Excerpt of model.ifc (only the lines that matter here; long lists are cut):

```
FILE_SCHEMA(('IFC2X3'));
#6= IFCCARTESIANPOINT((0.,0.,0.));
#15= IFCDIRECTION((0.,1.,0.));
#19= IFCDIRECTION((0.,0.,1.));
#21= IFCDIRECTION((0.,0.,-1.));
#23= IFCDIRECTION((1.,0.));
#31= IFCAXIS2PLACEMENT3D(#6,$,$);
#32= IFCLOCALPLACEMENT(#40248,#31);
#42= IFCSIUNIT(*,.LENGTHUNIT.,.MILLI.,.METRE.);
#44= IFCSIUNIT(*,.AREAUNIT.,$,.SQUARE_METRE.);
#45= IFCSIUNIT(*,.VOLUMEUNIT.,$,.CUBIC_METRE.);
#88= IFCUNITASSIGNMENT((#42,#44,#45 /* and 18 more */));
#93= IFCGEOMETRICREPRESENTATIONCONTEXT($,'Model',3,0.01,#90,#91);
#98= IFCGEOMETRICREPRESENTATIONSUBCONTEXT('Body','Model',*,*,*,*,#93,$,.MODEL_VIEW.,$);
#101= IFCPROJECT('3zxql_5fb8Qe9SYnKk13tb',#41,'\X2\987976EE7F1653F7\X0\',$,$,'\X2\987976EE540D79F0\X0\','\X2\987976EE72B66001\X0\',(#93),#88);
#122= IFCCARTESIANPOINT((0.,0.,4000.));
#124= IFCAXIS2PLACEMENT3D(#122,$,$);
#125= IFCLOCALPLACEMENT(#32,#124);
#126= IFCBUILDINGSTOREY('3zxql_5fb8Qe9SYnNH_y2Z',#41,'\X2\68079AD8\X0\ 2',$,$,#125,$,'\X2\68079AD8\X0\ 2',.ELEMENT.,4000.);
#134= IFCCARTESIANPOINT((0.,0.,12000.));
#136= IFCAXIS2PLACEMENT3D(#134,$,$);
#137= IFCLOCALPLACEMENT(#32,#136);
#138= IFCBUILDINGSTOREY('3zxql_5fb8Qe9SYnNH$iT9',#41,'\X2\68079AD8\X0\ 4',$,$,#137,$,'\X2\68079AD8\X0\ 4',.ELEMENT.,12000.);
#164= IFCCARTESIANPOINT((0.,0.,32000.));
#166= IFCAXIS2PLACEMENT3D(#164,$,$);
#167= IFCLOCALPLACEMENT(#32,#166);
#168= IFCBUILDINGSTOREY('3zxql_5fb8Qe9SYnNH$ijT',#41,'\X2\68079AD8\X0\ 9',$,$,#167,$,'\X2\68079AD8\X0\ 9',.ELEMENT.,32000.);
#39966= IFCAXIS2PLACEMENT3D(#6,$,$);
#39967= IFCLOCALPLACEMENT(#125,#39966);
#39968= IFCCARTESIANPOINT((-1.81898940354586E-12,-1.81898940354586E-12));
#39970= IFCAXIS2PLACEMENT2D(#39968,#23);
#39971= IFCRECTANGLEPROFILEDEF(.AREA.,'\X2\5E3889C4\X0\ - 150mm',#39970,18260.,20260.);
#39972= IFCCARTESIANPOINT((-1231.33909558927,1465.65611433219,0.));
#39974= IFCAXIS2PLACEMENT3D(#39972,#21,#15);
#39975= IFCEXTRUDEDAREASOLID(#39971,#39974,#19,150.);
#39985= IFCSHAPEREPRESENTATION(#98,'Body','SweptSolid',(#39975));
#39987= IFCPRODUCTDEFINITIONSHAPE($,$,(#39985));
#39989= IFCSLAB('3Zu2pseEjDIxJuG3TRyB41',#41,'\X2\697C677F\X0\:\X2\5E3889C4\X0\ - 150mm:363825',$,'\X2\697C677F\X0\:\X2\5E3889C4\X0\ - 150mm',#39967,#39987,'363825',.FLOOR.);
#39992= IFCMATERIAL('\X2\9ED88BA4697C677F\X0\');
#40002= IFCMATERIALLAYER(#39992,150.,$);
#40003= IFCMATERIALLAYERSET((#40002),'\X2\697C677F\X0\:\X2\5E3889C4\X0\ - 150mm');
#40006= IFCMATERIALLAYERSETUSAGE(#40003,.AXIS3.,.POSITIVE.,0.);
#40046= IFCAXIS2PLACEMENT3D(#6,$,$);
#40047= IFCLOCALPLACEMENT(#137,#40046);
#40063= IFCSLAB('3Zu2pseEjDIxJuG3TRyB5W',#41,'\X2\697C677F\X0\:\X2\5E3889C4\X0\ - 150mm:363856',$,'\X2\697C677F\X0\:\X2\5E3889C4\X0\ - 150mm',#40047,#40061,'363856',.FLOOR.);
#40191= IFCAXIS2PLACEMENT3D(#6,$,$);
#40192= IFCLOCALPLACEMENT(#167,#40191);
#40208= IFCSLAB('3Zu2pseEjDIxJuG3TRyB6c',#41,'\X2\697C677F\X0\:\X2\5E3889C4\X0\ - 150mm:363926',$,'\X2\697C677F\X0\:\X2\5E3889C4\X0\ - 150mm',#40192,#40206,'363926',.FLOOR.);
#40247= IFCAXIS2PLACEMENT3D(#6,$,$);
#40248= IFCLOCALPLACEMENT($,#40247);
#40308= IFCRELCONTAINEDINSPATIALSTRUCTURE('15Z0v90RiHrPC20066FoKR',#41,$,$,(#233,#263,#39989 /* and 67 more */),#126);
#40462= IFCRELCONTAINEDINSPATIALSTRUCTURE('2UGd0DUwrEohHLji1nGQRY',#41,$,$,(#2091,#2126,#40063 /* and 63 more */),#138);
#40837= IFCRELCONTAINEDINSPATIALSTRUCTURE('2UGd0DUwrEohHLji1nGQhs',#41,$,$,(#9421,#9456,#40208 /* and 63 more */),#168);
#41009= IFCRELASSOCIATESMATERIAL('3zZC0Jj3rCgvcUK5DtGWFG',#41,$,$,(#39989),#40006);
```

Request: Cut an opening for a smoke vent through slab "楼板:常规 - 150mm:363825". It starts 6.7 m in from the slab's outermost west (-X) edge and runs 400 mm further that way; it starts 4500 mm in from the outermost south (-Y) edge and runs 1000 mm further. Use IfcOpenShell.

```python
import numpy as np
import ifcopenshell
import ifcopenshell.api.feature
import ifcopenshell.api.geometry
import ifcopenshell.api.root
import ifcopenshell.geom
import ifcopenshell.util.placement
import ifcopenshell.util.representation
import ifcopenshell.util.shape
import ifcopenshell.util.unit

model = ifcopenshell.open("model.ifc")
unit_scale = ifcopenshell.util.unit.calculate_unit_scale(model)
settings = ifcopenshell.geom.settings()


def volume(element):
    """Net volume in cubic metres, openings subtracted."""
    shape = ifcopenshell.geom.create_shape(settings, element)
    return ifcopenshell.util.shape.get_volume(shape.geometry)


slab = model.by_guid("3Zu2pseEjDIxJuG3TRyB41")
before = volume(slab)

# Extent in the slab's own axes, in metres. The edges named are its -X and -Y sides.
slab_shape = ifcopenshell.geom.create_shape(settings, slab)
vertices = ifcopenshell.util.shape.get_vertices(slab_shape.geometry)
x_min, y_min, bottom = vertices.min(axis=0)
top = vertices[:, 2].max()

opening = ifcopenshell.api.root.create_entity(model, ifc_class="IfcOpeningElement", name="Smoke vent opening")
context = ifcopenshell.util.representation.get_context(model, "Model", "Body", "MODEL_VIEW")
width, depth = 0.4, 1
outline = [(0.0, 0.0), (width, 0.0), (width, depth), (0.0, depth), (0.0, 0.0)]
# Overshoot both faces by 50 mm so the cut is clean.
shape = ifcopenshell.api.geometry.add_slab_representation(
    model, context=context, depth=top - bottom + 0.1, polyline=outline
)
ifcopenshell.api.geometry.assign_representation(model, product=opening, representation=shape)

matrix = ifcopenshell.util.placement.get_local_placement(slab.ObjectPlacement)
matrix[:, 3] = matrix @ np.append(np.array([x_min + 6.7, y_min + 4.5, bottom - 0.05]) / unit_scale, 1.0)
ifcopenshell.api.geometry.edit_object_placement(model, product=opening, matrix=matrix, is_si=False)
ifcopenshell.api.feature.add_feature(model, feature=opening, element=slab)

after = volume(slab)

print(f"slab volume {before:.3f} -> {after:.3f} m3")

model.write("model_updated.ifc")
```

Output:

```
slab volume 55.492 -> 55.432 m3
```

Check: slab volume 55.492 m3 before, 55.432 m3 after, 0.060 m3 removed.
